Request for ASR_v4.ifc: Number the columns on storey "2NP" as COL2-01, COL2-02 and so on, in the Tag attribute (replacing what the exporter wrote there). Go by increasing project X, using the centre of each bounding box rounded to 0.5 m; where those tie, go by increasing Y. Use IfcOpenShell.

First a look at what the model holds.

```python
import ifcopenshell
import ifcopenshell.util.element
import ifcopenshell.util.placement

model = ifcopenshell.open("ASR_v4.ifc")
print(model.schema)
storey = next(s for s in model.by_type("IfcBuildingStorey") if s.Name == "2NP")
columns = [e for e in ifcopenshell.util.element.get_decomposition(storey) if e.is_a("IfcColumn")]
for e in sorted(columns, key=lambda e: e.id()):
    origin = ifcopenshell.util.placement.get_local_placement(e.ObjectPlacement)[:3, 3]
    print(e.id(), e.Tag, e.Name, origin.round(2) + 0.0, sep=" | ")
```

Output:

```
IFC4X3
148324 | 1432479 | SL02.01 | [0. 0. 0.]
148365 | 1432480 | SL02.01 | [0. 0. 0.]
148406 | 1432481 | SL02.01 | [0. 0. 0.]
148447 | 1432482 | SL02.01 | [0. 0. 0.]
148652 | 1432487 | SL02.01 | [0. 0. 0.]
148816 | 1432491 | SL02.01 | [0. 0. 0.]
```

```python
import ifcopenshell
import ifcopenshell.geom
import ifcopenshell.util.element
import ifcopenshell.util.shape

model = ifcopenshell.open("ASR_v4.ifc")
settings = ifcopenshell.geom.settings()
settings.set("use-world-coords", True)


def centre(element):
    shape = ifcopenshell.geom.create_shape(settings, element)
    return ifcopenshell.util.shape.get_bbox_centroid(shape.geometry)


storey = next(s for s in model.by_type("IfcBuildingStorey") if s.Name == "2NP")
columns = [e for e in ifcopenshell.util.element.get_decomposition(storey) if e.is_a("IfcColumn")]

# Insertion points can sit at a corner or the storey origin, so sort by the geometry (in metres).
centres = {e: centre(e) for e in columns}
columns.sort(key=lambda e: (round(centres[e][0] / 0.5), centres[e][1]))

for i, e in enumerate(columns, start=1):
    number = f"COL2-{i:02d}"
    e.Tag = number
    print(e.id(), number)

model.write("ASR_v4_rev.ifc")
```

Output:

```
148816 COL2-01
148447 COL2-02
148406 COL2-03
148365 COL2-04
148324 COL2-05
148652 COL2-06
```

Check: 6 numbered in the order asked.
